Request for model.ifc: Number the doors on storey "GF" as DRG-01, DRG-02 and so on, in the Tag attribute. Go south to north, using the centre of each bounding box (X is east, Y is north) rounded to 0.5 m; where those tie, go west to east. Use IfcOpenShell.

First a look at what the model holds.

```python
import ifcopenshell
import ifcopenshell.util.element
import ifcopenshell.util.placement

model = ifcopenshell.open("model.ifc")
print(model.schema)
storey = next(s for s in model.by_type("IfcBuildingStorey") if s.Name == "GF")
doors = [e for e in ifcopenshell.util.element.get_decomposition(storey) if e.is_a("IfcDoor")]
for e in sorted(doors, key=lambda e: e.id()):
    origin = ifcopenshell.util.placement.get_local_placement(e.ObjectPlacement)[:3, 3]
    print(e.id(), e.Tag, e.Name, origin.round(2) + 0.0, sep=" | ")
```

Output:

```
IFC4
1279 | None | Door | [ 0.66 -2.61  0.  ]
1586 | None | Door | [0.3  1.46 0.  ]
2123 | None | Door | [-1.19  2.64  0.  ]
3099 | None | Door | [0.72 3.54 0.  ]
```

```python
import ifcopenshell
import ifcopenshell.geom
import ifcopenshell.util.element
import ifcopenshell.util.shape

model = ifcopenshell.open("model.ifc")
settings = ifcopenshell.geom.settings()
settings.set("use-world-coords", True)


def centre(element):
    shape = ifcopenshell.geom.create_shape(settings, element)
    return ifcopenshell.util.shape.get_bbox_centroid(shape.geometry)


storey = next(s for s in model.by_type("IfcBuildingStorey") if s.Name == "GF")
doors = [e for e in ifcopenshell.util.element.get_decomposition(storey) if e.is_a("IfcDoor")]

# Insertion points can sit at a corner or the storey origin, so sort by the geometry (in metres).
centres = {e: centre(e) for e in doors}
doors.sort(key=lambda e: (round(centres[e][1] / 0.5), centres[e][0]))

for i, e in enumerate(doors, start=1):
    number = f"DRG-{i:02d}"
    e.Tag = number
    print(e.id(), number)

model.write("model_rev.ifc")
```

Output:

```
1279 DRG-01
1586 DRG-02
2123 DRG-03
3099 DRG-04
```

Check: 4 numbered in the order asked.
